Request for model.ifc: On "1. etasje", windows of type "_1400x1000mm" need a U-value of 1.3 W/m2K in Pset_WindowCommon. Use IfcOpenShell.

First a look at what the model holds.

```python
import ifcopenshell
import ifcopenshell.util.element

model = ifcopenshell.open("model.ifc")
print(model.schema)
storey = next(s for s in model.by_type("IfcBuildingStorey") if s.Name == "1. etasje")
windows = [e for e in ifcopenshell.util.element.get_decomposition(storey) if e.is_a("IfcWindow")]
seen = {}
for e in windows:
    element_type = ifcopenshell.util.element.get_type(e)
    key = (element_type.Name if element_type != e and element_type else None, ifcopenshell.util.element.get_pset(e, "Pset_WindowCommon", "ThermalTransmittance"))
    seen[key] = seen.get(key, 0) + 1
for (name, value), count in sorted(seen.items(), key=str):
    print(count, "x", name, "|", value)
```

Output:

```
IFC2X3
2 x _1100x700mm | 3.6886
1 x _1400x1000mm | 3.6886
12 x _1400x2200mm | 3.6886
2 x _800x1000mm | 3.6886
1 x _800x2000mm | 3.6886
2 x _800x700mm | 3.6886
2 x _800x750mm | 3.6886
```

```python
import ifcopenshell
import ifcopenshell.api.pset
import ifcopenshell.util.element

model = ifcopenshell.open("model.ifc")

storey = next(s for s in model.by_type("IfcBuildingStorey") if s.Name == "1. etasje")
windows = [e for e in ifcopenshell.util.element.get_decomposition(storey) if e.is_a("IfcWindow")]

count = 0
for e in windows:
    element_type = ifcopenshell.util.element.get_type(e)
    if element_type in (None, e) or element_type.Name != "_1400x1000mm":
        continue
    # add_pset returns the element's existing set when there is one.
    pset = ifcopenshell.api.pset.add_pset(model, product=e, name="Pset_WindowCommon")
    ifcopenshell.api.pset.edit_pset(model, pset=pset, properties={"ThermalTransmittance": 1.3})
    count += 1

print(count, "windows updated")

model.write("model_rev.ifc")
```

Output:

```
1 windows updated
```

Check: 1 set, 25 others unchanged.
